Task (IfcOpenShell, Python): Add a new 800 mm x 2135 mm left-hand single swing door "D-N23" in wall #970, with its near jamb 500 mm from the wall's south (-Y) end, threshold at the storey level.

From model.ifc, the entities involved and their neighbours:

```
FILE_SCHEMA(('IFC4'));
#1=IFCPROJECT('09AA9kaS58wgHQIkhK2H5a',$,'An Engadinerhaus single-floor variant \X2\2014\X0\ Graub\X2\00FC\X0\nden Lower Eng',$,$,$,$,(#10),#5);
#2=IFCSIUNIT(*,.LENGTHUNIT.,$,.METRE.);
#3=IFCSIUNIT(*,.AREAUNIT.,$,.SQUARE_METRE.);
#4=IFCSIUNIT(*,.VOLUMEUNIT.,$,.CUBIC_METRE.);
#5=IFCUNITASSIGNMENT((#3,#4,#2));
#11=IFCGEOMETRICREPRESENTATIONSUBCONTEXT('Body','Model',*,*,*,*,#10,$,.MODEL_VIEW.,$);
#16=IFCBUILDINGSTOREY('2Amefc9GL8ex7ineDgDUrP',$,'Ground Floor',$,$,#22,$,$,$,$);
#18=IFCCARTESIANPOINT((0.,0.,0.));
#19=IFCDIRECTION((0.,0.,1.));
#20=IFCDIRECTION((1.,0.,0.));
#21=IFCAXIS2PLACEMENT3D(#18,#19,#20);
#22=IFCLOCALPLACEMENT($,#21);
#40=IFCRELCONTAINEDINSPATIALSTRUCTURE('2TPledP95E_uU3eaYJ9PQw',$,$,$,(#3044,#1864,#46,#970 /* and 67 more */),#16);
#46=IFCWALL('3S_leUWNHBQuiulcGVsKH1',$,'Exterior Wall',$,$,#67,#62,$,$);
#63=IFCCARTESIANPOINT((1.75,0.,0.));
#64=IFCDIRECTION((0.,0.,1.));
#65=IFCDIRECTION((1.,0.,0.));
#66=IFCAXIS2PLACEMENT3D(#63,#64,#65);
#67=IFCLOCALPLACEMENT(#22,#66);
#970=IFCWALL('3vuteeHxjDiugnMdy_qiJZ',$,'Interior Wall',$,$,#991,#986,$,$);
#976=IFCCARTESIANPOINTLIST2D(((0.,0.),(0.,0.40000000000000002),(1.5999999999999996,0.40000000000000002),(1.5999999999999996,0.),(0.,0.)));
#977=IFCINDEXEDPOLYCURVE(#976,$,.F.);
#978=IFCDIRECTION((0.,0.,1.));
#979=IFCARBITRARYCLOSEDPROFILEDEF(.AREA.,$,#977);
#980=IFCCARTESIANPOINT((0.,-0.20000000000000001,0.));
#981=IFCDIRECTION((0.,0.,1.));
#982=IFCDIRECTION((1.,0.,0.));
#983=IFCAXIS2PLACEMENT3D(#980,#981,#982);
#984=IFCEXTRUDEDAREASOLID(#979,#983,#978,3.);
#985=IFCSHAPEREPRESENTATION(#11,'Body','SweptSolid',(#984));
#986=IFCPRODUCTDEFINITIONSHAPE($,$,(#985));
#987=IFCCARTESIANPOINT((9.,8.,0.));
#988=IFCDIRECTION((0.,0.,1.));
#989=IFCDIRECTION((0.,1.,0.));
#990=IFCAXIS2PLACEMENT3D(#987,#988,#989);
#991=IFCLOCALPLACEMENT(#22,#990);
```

```python
import numpy as np
import ifcopenshell
import ifcopenshell.api.feature
import ifcopenshell.api.geometry
import ifcopenshell.api.root
import ifcopenshell.api.spatial
import ifcopenshell.geom
import ifcopenshell.util.element
import ifcopenshell.util.placement
import ifcopenshell.util.representation
import ifcopenshell.util.shape
import ifcopenshell.util.unit

model = ifcopenshell.open("model.ifc")
unit_scale = ifcopenshell.util.unit.calculate_unit_scale(model)
settings = ifcopenshell.geom.settings()


def volume(element):
    """Net volume in cubic metres, openings subtracted."""
    shape = ifcopenshell.geom.create_shape(settings, element)
    return ifcopenshell.util.shape.get_volume(shape.geometry)


wall = model.by_guid("3vuteeHxjDiugnMdy_qiJZ")
storey = ifcopenshell.util.element.get_container(wall, ifc_class="IfcBuildingStorey")
context = ifcopenshell.util.representation.get_context(model, "Model", "Body", "MODEL_VIEW")
before = volume(wall)

width, height, from_end, sill = 0.8, 2.135, 0.5, 0.0  # metres

# The wall runs along its own X axis, and the end named is its -X end.
wall_shape = ifcopenshell.geom.create_shape(settings, wall)
x, y, z = ifcopenshell.util.shape.get_vertices(wall_shape.geometry).T
start = x.min() + from_end
face, thickness = float(y.min()), float(y.max() - y.min())
wall_matrix = ifcopenshell.util.placement.get_local_placement(wall.ObjectPlacement)
level = ifcopenshell.util.placement.get_local_placement(storey.ObjectPlacement)[2, 3]


def in_wall(x, y):
    """Placement at x, y metres in the wall's axes, at sill height."""
    matrix = wall_matrix.copy()
    matrix[:, 3] = wall_matrix @ np.array([x / unit_scale, y / unit_scale, 0.0, 1.0])
    matrix[2, 3] = level + sill / unit_scale
    return matrix


# Opening: a box that overshoots both wall faces by 50 mm.
opening = ifcopenshell.api.root.create_entity(model, ifc_class="IfcOpeningElement", predefined_type="OPENING")
box = ifcopenshell.api.geometry.add_wall_representation(
    model, context=context, length=width, height=height, thickness=thickness + 0.1
)
ifcopenshell.api.geometry.assign_representation(model, product=opening, representation=box)
ifcopenshell.api.geometry.edit_object_placement(model, product=opening, matrix=in_wall(start, face - 0.05), is_si=False)
ifcopenshell.api.feature.add_feature(model, feature=opening, element=wall)

door = ifcopenshell.api.root.create_entity(model, ifc_class="IfcDoor", name="D-N23", predefined_type="DOOR")
door.OverallWidth, door.OverallHeight = width / unit_scale, height / unit_scale
door.OperationType = "SINGLE_SWING_LEFT"
body = ifcopenshell.api.geometry.add_door_representation(
    model,
    context=context,
    overall_width=door.OverallWidth,
    overall_height=door.OverallHeight,
    operation_type="SINGLE_SWING_LEFT",
    lining_properties={"LiningDepth": thickness / unit_scale, "ThresholdDepth": thickness / unit_scale},
)
ifcopenshell.api.geometry.assign_representation(model, product=door, representation=body)
ifcopenshell.api.spatial.assign_container(model, products=[door], relating_structure=storey)
ifcopenshell.api.feature.add_filling(model, opening=opening, element=door)

# The lining spans the wall, so the door starts at the wall face.
ifcopenshell.api.geometry.edit_object_placement(model, product=door, matrix=in_wall(start, face), is_si=False)

after = volume(wall)

print(f"wall volume {before:.3f} -> {after:.3f} m3")

model.write("model_updated.ifc")
```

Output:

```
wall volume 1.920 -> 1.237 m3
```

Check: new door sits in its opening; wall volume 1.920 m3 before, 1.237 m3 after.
